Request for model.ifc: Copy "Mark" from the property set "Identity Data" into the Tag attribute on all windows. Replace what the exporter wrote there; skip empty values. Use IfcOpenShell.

First a look at what the model holds.

```python
import ifcopenshell
import ifcopenshell.util.element

model = ifcopenshell.open("model.ifc")
print(model.schema)
windows = model.by_type("IfcWindow")
print(len(windows), "windows")
for e in windows[:8]:
    source = ifcopenshell.util.element.get_pset(e, "Identity Data", "Mark")
    target = e.Tag
    print(e.id(), repr(source), repr(target), sep=" | ")
```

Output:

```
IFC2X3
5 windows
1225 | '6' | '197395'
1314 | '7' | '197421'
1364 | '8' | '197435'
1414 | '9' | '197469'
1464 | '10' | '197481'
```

```python
import ifcopenshell
import ifcopenshell.util.element

model = ifcopenshell.open("model.ifc")

count = 0
for e in model.by_type("IfcWindow"):
    value = ifcopenshell.util.element.get_pset(e, "Identity Data", "Mark")
    current = e.Tag
    if not value or not value.strip() or current == value:
        continue
    e.Tag = value
    count += 1

print(count, "windows updated")

model.write("model-out.ifc")
```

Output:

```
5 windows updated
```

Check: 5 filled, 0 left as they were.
